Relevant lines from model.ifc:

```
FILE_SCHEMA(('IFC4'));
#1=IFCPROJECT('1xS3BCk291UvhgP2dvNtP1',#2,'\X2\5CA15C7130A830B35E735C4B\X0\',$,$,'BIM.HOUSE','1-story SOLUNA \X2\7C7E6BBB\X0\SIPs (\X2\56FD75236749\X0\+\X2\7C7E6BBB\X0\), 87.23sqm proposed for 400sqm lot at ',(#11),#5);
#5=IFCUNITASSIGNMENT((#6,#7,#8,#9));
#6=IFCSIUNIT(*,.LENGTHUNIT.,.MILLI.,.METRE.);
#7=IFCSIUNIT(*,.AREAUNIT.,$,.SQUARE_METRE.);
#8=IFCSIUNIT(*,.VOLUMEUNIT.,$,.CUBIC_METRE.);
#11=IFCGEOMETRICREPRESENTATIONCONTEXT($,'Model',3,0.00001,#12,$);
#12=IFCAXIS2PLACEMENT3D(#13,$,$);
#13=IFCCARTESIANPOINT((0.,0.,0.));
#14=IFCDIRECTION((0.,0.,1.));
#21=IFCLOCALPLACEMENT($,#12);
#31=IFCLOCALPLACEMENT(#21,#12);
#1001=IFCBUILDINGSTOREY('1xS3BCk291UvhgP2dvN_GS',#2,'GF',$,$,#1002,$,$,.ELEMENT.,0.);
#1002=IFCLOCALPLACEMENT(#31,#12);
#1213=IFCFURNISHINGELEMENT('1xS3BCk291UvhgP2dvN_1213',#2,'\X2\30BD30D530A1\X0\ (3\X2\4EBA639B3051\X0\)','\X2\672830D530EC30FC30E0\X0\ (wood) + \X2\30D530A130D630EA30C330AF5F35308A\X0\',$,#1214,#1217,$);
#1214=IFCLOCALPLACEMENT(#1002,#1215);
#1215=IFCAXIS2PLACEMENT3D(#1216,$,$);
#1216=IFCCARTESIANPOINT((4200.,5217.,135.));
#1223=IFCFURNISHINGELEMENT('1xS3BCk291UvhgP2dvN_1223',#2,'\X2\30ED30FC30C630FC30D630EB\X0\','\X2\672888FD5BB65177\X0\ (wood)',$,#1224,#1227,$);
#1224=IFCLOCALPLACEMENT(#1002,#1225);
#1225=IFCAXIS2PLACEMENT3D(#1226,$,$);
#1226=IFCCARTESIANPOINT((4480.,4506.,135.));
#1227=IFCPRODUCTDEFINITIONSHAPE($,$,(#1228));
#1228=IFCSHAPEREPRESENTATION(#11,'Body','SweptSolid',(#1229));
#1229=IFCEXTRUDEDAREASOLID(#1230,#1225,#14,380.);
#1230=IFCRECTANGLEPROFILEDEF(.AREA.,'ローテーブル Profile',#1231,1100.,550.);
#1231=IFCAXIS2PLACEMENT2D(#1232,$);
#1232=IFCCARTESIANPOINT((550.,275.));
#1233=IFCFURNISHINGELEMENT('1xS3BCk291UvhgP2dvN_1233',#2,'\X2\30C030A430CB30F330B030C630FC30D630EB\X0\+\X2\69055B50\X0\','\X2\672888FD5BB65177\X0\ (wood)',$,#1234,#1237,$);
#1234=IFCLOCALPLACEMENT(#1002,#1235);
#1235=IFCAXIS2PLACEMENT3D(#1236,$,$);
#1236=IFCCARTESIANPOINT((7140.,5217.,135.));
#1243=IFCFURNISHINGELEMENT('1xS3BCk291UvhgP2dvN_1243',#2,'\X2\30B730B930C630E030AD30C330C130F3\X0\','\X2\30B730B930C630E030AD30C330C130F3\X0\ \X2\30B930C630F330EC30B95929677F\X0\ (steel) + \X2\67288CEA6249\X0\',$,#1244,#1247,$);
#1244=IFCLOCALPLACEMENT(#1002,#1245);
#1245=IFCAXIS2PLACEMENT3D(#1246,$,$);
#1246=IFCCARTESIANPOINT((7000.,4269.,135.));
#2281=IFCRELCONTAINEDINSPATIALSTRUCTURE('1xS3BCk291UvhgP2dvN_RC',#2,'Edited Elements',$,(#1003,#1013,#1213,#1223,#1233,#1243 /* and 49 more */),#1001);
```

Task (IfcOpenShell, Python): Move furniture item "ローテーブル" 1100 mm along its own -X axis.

```python
import ifcopenshell
import ifcopenshell.api.geometry
import ifcopenshell.util.placement

model = ifcopenshell.open("model.ifc")

item = model.by_guid("1xS3BCk291UvhgP2dvN_1223")
matrix = ifcopenshell.util.placement.get_local_placement(item.ObjectPlacement)
matrix[:3, 3] -= matrix[:3, 0] * 1100.0
ifcopenshell.api.geometry.edit_object_placement(model, product=item, matrix=matrix, is_si=False)

print(ifcopenshell.util.placement.get_local_placement(item.ObjectPlacement).round(3) + 0.0)

model.write("model_edited.ifc")
```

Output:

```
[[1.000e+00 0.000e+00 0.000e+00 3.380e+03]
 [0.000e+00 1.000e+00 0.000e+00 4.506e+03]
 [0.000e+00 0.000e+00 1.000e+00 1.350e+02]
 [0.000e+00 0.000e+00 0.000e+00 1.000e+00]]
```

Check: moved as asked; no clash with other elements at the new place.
